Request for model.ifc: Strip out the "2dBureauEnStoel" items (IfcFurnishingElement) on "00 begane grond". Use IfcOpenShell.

First a look at what the model holds.

```python
import ifcopenshell
import ifcopenshell.util.element

model = ifcopenshell.open("model.ifc")
print(model.schema)
storey = next(s for s in model.by_type("IfcBuildingStorey") if s.Name == "00 begane grond")
furniture = [e for e in ifcopenshell.util.element.get_decomposition(storey) if e.is_a("IfcFurnishingElement")]
seen = {}
for e in furniture:
    element_type = ifcopenshell.util.element.get_type(e)
    name = element_type.Name if element_type not in (None, e) else None
    seen[name] = seen.get(name, 0) + 1
for name, count in sorted(seen.items(), key=str):
    print(count, "x", name)
```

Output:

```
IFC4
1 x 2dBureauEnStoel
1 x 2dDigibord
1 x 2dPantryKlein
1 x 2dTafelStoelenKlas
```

```python
import ifcopenshell
import ifcopenshell.api.root
import ifcopenshell.util.element

model = ifcopenshell.open("model.ifc")

storey = next(s for s in model.by_type("IfcBuildingStorey") if s.Name == "00 begane grond")
furniture = [e for e in ifcopenshell.util.element.get_decomposition(storey) if e.is_a("IfcFurnishingElement")]
targets = [e for e in furniture if (t := ifcopenshell.util.element.get_type(e)) not in (None, e) and t.Name == "2dBureauEnStoel"]

for e in targets:
    ifcopenshell.api.root.remove_product(model, product=e)
print(len(targets), "removed")

model.write("model-out.ifc")
```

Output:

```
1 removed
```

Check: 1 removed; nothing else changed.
